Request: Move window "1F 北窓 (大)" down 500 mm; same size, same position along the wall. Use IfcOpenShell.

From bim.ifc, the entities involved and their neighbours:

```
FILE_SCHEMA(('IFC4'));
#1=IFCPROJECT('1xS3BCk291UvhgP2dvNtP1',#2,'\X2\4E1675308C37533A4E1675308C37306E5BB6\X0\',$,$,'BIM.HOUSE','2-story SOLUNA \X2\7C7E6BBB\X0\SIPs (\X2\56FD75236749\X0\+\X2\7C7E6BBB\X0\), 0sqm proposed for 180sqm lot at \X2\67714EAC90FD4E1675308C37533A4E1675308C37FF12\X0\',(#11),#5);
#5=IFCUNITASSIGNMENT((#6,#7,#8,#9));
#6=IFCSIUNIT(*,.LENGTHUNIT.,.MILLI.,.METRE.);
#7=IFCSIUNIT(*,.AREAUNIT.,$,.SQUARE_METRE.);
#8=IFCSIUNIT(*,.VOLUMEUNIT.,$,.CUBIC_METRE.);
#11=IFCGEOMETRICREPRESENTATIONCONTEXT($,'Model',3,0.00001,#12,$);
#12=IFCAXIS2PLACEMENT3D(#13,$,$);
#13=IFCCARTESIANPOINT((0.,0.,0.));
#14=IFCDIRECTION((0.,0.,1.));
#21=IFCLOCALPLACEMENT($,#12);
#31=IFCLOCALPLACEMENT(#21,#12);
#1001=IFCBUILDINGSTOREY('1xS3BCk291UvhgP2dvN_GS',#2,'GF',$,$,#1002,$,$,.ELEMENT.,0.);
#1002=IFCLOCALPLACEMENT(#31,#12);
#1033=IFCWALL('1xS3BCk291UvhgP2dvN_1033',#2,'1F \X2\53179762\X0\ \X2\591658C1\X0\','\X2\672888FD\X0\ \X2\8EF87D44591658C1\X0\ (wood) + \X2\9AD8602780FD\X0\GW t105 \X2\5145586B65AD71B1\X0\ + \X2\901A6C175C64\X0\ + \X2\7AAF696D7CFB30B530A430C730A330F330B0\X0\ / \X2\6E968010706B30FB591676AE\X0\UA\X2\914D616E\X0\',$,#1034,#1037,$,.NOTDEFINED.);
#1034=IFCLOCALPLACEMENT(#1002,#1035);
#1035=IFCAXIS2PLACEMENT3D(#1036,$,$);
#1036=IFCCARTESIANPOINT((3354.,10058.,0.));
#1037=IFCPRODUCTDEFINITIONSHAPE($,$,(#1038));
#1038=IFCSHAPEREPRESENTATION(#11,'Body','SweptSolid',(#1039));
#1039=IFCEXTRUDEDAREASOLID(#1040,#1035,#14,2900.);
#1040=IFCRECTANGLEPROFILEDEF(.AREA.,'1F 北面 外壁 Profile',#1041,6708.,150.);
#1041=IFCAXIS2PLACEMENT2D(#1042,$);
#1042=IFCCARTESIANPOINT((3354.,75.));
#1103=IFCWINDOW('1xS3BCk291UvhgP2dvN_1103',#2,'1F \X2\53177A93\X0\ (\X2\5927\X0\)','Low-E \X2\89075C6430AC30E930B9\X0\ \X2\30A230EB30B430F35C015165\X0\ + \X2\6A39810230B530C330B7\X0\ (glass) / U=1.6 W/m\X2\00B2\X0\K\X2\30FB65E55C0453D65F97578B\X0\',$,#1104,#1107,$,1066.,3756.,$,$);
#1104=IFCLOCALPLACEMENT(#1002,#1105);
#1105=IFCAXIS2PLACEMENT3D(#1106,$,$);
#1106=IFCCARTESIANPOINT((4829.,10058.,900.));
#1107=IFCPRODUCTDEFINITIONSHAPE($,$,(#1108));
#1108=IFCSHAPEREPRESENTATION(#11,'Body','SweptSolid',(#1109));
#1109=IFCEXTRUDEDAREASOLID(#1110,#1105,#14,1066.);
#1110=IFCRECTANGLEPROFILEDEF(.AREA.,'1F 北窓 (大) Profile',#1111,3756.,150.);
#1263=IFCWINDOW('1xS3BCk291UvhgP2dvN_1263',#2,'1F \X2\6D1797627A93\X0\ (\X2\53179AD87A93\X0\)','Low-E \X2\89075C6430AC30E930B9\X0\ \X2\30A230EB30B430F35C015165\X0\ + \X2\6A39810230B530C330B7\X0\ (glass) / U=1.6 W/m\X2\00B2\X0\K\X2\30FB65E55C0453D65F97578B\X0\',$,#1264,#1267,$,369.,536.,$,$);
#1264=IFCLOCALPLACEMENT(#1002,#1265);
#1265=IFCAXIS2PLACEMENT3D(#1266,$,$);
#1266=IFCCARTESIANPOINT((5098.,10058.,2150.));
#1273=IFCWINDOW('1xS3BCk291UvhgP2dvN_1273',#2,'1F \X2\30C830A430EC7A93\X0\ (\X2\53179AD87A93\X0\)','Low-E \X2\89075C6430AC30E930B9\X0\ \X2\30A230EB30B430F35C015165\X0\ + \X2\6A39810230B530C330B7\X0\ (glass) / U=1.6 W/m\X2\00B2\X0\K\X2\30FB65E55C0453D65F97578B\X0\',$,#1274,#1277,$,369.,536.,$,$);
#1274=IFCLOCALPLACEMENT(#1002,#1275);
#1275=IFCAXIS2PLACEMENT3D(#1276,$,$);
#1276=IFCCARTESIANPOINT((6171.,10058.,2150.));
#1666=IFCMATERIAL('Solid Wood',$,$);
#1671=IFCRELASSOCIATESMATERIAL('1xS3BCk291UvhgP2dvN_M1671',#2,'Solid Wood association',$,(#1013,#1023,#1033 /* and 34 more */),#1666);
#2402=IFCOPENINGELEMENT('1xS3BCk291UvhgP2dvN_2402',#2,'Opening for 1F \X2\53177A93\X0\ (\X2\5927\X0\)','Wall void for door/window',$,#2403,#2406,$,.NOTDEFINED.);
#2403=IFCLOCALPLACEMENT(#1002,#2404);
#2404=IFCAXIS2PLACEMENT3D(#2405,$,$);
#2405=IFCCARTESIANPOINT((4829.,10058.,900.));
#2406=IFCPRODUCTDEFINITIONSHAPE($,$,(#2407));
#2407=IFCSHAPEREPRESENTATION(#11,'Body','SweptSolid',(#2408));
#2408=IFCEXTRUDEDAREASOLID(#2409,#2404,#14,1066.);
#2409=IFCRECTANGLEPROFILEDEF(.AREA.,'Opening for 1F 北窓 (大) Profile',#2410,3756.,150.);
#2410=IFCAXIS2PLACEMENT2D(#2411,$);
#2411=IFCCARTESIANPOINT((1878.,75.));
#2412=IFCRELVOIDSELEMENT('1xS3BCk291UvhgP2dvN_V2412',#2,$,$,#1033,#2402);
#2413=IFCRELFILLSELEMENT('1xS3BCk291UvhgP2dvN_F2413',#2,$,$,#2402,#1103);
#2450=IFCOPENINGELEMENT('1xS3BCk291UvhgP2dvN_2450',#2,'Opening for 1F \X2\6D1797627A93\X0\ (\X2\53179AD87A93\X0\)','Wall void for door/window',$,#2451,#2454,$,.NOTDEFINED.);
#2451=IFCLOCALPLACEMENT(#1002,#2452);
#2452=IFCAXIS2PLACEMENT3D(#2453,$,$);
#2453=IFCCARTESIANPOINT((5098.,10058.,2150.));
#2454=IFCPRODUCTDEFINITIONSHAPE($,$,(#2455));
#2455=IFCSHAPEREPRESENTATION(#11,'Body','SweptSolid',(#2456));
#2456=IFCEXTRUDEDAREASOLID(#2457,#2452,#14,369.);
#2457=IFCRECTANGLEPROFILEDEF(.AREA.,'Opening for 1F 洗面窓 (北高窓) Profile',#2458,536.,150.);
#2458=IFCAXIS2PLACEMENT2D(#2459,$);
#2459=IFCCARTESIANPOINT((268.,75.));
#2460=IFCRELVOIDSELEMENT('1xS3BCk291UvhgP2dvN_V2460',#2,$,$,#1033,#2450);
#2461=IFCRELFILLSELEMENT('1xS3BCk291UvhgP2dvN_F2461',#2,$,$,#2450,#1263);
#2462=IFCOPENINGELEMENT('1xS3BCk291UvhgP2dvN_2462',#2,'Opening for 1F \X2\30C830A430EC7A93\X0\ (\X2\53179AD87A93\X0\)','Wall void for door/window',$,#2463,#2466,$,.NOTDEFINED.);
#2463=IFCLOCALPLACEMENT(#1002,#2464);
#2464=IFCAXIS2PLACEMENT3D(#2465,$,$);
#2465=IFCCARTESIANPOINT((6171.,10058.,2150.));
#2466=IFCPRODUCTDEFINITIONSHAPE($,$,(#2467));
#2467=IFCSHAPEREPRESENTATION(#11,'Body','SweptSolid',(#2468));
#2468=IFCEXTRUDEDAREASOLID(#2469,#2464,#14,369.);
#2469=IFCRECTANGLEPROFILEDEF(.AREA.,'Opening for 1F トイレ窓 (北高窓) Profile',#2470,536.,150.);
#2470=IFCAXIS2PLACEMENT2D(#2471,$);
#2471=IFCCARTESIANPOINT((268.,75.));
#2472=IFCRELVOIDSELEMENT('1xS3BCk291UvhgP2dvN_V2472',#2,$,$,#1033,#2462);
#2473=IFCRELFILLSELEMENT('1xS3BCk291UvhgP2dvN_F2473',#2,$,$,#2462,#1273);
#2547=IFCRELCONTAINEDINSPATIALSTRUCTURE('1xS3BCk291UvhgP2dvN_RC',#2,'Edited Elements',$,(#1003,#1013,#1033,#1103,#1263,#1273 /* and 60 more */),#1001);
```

```python
import numpy as np
import ifcopenshell
import ifcopenshell.api.geometry
import ifcopenshell.util.placement
import ifcopenshell.util.unit

model = ifcopenshell.open("bim.ifc")
unit_scale = ifcopenshell.util.unit.calculate_unit_scale(model)

window = model.by_guid("1xS3BCk291UvhgP2dvN_1103")
opening = window.FillsVoids[0].RelatingOpeningElement
dz = -500.0

shift = np.array([0.0, 0.0, dz])
# The window is not placed relative to its opening, so move both.
for product in (opening, window):
    matrix = ifcopenshell.util.placement.get_local_placement(product.ObjectPlacement)
    matrix[:3, 3] += shift
    ifcopenshell.api.geometry.edit_object_placement(model, product=product, matrix=matrix, is_si=False)

print(f"moved by {dz * unit_scale:+.3f} m")

model.write("bim_edited.ifc")
```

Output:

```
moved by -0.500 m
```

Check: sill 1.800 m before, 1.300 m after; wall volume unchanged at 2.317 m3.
